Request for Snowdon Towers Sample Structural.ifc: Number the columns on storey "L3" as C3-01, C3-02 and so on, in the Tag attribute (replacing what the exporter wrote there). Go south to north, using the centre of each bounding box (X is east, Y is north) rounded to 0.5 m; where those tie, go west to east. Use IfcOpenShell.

First a look at what the model holds.

```python
import ifcopenshell
import ifcopenshell.util.element
import ifcopenshell.util.placement

model = ifcopenshell.open("Snowdon Towers Sample Structural.ifc")
print(model.schema)
storey = next(s for s in model.by_type("IfcBuildingStorey") if s.Name == "L3")
columns = [e for e in ifcopenshell.util.element.get_decomposition(storey) if e.is_a("IfcColumn")]
for e in sorted(columns, key=lambda e: e.id()):
    origin = ifcopenshell.util.placement.get_local_placement(e.ObjectPlacement)[:3, 3]
    print(e.id(), e.Tag, e.Name, origin.round(2) + 0.0, sep=" | ")
```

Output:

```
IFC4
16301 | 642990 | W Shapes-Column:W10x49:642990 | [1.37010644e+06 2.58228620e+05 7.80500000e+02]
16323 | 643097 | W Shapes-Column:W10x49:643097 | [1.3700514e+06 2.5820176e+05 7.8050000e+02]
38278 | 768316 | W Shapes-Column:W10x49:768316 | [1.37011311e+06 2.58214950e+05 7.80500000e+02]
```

```python
import ifcopenshell
import ifcopenshell.geom
import ifcopenshell.util.element
import ifcopenshell.util.shape

model = ifcopenshell.open("Snowdon Towers Sample Structural.ifc")
settings = ifcopenshell.geom.settings()
settings.set("use-world-coords", True)


def centre(element):
    shape = ifcopenshell.geom.create_shape(settings, element)
    return ifcopenshell.util.shape.get_bbox_centroid(shape.geometry)


storey = next(s for s in model.by_type("IfcBuildingStorey") if s.Name == "L3")
columns = [e for e in ifcopenshell.util.element.get_decomposition(storey) if e.is_a("IfcColumn")]

# Insertion points can sit at a corner or the storey origin, so sort by the geometry (in metres).
centres = {e: centre(e) for e in columns}
columns.sort(key=lambda e: (round(centres[e][1] / 0.5), centres[e][0]))

for i, e in enumerate(columns, start=1):
    number = f"C3-{i:02d}"
    e.Tag = number
    print(e.id(), number)

model.write("Snowdon Towers Sample Structural_v2.ifc")
```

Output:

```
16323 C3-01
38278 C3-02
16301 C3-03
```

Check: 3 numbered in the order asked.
